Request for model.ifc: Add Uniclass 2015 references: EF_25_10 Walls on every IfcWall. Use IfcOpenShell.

First a look at what the model holds.

```python
import ifcopenshell

model = ifcopenshell.open("model.ifc")
print(model.schema)
print("classifications:", [c.Name for c in model.by_type("IfcClassification")])
for ifc_class in ("IfcDoor", "IfcRoof", "IfcStair", "IfcWall", "IfcWindow"):
    print(ifc_class, len(model.by_type(ifc_class)))
```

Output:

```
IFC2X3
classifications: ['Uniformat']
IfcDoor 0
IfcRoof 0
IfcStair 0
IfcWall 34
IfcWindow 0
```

```python
import ifcopenshell
import ifcopenshell.api.classification

model = ifcopenshell.open("model.ifc")

# IFC2X3 requires Source and Edition and has no link from the project to the system.
system = model.create_entity("IfcClassification", Source="NBS", Edition="2015", Name="Uniclass 2015")

codes = {
    "IfcWall": ("EF_25_10", "Walls"),
}
for ifc_class, (code, name) in codes.items():
    products = model.by_type(ifc_class)
    ifcopenshell.api.classification.add_reference(
        model, products=products, classification=system, identification=code, name=name
    )
    print(code, len(products))

model.write("model_v2.ifc")
```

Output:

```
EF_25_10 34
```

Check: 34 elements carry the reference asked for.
